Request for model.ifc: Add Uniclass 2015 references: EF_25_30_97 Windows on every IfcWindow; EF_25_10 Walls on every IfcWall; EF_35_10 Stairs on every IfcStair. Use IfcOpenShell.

First a look at what the model holds.

```python
import ifcopenshell

model = ifcopenshell.open("model.ifc")
print(model.schema)
print("classifications:", [c.Name for c in model.by_type("IfcClassification")])
for ifc_class in ("IfcDoor", "IfcRoof", "IfcStair", "IfcWall", "IfcWindow"):
    print(ifc_class, len(model.by_type(ifc_class)))
```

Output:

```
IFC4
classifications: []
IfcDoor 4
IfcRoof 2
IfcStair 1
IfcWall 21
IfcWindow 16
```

```python
import ifcopenshell
import ifcopenshell.api.classification

model = ifcopenshell.open("model.ifc")

system = ifcopenshell.api.classification.add_classification(model, classification="Uniclass 2015")

codes = {
    "IfcWindow": ("EF_25_30_97", "Windows"),
    "IfcWall": ("EF_25_10", "Walls"),
    "IfcStair": ("EF_35_10", "Stairs"),
}
for ifc_class, (code, name) in codes.items():
    products = model.by_type(ifc_class)
    ifcopenshell.api.classification.add_reference(
        model, products=products, classification=system, identification=code, name=name
    )
    print(code, len(products))

model.write("model_rev.ifc")
```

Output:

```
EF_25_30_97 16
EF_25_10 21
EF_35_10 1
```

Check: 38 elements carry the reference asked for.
